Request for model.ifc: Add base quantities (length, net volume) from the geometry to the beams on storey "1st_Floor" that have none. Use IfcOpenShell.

First a look at what the model holds.

```python
import ifcopenshell
import ifcopenshell.util.element
import ifcopenshell.util.unit

model = ifcopenshell.open("model.ifc")
print(model.schema)
for unit_type in ("LENGTHUNIT", "AREAUNIT", "VOLUMEUNIT"):
    print(unit_type, ifcopenshell.util.unit.calculate_unit_scale(model, unit_type))
storey = next(s for s in model.by_type("IfcBuildingStorey") if s.Name == "1st_Floor")
beams = [e for e in ifcopenshell.util.element.get_decomposition(storey) if e.is_a("IfcBeam")]
for e in sorted(beams, key=lambda e: e.id()):
    print(e.id(), e.is_a(), e.Name, list(ifcopenshell.util.element.get_psets(e, qtos_only=True)), sep=" | ")
```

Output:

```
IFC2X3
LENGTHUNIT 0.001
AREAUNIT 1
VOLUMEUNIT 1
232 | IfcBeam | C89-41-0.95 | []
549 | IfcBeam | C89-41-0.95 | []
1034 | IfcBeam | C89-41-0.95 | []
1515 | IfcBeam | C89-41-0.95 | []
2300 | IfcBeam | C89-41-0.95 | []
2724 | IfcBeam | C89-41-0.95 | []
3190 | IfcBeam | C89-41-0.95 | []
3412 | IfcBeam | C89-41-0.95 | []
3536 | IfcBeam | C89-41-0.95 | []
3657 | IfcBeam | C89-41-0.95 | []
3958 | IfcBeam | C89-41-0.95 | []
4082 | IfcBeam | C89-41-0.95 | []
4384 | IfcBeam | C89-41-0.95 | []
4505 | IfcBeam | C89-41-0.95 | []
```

```python
import ifcopenshell
import ifcopenshell.api.pset
import ifcopenshell.geom
import ifcopenshell.util.element
import ifcopenshell.util.shape
import ifcopenshell.util.unit

model = ifcopenshell.open("model.ifc")
unit_scale = ifcopenshell.util.unit.calculate_unit_scale(model)
volume_scale = ifcopenshell.util.unit.calculate_unit_scale(model, "VOLUMEUNIT")
settings = ifcopenshell.geom.settings()

storey = next(s for s in model.by_type("IfcBuildingStorey") if s.Name == "1st_Floor")
beams = [e for e in ifcopenshell.util.element.get_decomposition(storey) if e.is_a("IfcBeam")]

for e in sorted(beams, key=lambda e: e.id()):
    if ifcopenshell.util.element.get_psets(e, qtos_only=True, should_inherit=False):
        continue
    # Geometry comes back in metres, in the element's own axes.
    shape = ifcopenshell.geom.create_shape(settings, e)
    values = {
        "Length": ifcopenshell.util.shape.get_max_xyz(shape.geometry) / unit_scale,
        "NetVolume": ifcopenshell.util.shape.get_volume(shape.geometry) / volume_scale,
    }
    qto = ifcopenshell.api.pset.add_qto(model, product=e, name="BaseQuantities")
    ifcopenshell.api.pset.edit_qto(model, qto=qto, properties=values)
    print(e.id(), {k: round(v, 3) for k, v in values.items()})

model.write("model_updated.ifc")
```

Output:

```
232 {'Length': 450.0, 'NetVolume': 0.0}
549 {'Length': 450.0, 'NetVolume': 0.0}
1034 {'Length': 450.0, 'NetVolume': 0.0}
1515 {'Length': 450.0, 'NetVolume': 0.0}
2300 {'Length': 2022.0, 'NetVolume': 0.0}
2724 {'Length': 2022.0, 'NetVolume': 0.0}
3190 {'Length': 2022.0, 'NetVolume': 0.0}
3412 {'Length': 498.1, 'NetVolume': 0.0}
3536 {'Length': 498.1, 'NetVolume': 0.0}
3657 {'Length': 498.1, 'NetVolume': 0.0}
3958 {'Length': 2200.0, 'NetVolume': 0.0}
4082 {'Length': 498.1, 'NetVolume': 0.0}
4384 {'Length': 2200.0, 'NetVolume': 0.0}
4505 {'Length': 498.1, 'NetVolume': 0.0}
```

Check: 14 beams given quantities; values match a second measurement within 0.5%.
